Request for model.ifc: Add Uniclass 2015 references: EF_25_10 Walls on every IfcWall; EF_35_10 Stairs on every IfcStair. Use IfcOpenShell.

First a look at what the model holds.

```python
import ifcopenshell

model = ifcopenshell.open("model.ifc")
print(model.schema)
print("classifications:", [c.Name for c in model.by_type("IfcClassification")])
for ifc_class in ("IfcDoor", "IfcRoof", "IfcStair", "IfcWall", "IfcWindow"):
    print(ifc_class, len(model.by_type(ifc_class)))
```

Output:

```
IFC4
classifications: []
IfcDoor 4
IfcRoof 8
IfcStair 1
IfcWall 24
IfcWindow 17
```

```python
import ifcopenshell
import ifcopenshell.api.classification

model = ifcopenshell.open("model.ifc")

system = ifcopenshell.api.classification.add_classification(model, classification="Uniclass 2015")

codes = {
    "IfcWall": ("EF_25_10", "Walls"),
    "IfcStair": ("EF_35_10", "Stairs"),
}
for ifc_class, (code, name) in codes.items():
    products = model.by_type(ifc_class)
    ifcopenshell.api.classification.add_reference(
        model, products=products, classification=system, identification=code, name=name
    )
    print(code, len(products))

model.write("model_v2.ifc")
```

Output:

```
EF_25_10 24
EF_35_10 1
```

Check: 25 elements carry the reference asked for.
